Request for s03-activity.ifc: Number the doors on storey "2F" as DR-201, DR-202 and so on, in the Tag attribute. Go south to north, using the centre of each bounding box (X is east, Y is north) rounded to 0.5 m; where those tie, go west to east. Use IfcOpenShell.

First a look at what the model holds.

```python
import ifcopenshell
import ifcopenshell.util.element
import ifcopenshell.util.placement

model = ifcopenshell.open("s03-activity.ifc")
print(model.schema)
storey = next(s for s in model.by_type("IfcBuildingStorey") if s.Name == "2F")
doors = [e for e in ifcopenshell.util.element.get_decomposition(storey) if e.is_a("IfcDoor")]
for e in sorted(doors, key=lambda e: e.id()):
    origin = ifcopenshell.util.placement.get_local_placement(e.ObjectPlacement)[:3, 3]
    print(e.id(), e.Tag, e.Name, origin.round(2) + 0.0, sep=" | ")
```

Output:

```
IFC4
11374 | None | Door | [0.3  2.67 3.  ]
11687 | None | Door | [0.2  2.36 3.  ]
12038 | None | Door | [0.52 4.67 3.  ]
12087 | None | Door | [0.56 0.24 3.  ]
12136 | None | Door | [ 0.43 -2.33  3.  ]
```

```python
import ifcopenshell
import ifcopenshell.geom
import ifcopenshell.util.element
import ifcopenshell.util.shape

model = ifcopenshell.open("s03-activity.ifc")
settings = ifcopenshell.geom.settings()
settings.set("use-world-coords", True)


def centre(element):
    shape = ifcopenshell.geom.create_shape(settings, element)
    return ifcopenshell.util.shape.get_bbox_centroid(shape.geometry)


storey = next(s for s in model.by_type("IfcBuildingStorey") if s.Name == "2F")
doors = [e for e in ifcopenshell.util.element.get_decomposition(storey) if e.is_a("IfcDoor")]

# Insertion points can sit at a corner or the storey origin, so sort by the geometry (in metres).
centres = {e: centre(e) for e in doors}
doors.sort(key=lambda e: (round(centres[e][1] / 0.5), centres[e][0]))

for i, e in enumerate(doors, start=1):
    number = f"DR-2{i:02d}"
    e.Tag = number
    print(e.id(), number)

model.write("s03-activity_v2.ifc")
```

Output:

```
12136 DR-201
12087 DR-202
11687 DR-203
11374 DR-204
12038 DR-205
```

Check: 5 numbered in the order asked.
